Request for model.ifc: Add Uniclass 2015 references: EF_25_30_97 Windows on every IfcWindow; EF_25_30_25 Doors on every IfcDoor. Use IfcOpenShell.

First a look at what the model holds.

```python
import ifcopenshell

model = ifcopenshell.open("model.ifc")
print(model.schema)
print("classifications:", [c.Name for c in model.by_type("IfcClassification")])
for ifc_class in ("IfcDoor", "IfcRoof", "IfcStair", "IfcWall", "IfcWindow"):
    print(ifc_class, len(model.by_type(ifc_class)))
```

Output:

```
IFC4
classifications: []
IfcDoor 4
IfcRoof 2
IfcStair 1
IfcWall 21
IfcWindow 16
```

```python
import ifcopenshell
import ifcopenshell.api.classification

model = ifcopenshell.open("model.ifc")

system = ifcopenshell.api.classification.add_classification(model, classification="Uniclass 2015")

codes = {
    "IfcWindow": ("EF_25_30_97", "Windows"),
    "IfcDoor": ("EF_25_30_25", "Doors"),
}
for ifc_class, (code, name) in codes.items():
    products = model.by_type(ifc_class)
    ifcopenshell.api.classification.add_reference(
        model, products=products, classification=system, identification=code, name=name
    )
    print(code, len(products))

model.write("model_v2.ifc")
```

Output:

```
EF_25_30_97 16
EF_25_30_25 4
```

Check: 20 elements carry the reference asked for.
